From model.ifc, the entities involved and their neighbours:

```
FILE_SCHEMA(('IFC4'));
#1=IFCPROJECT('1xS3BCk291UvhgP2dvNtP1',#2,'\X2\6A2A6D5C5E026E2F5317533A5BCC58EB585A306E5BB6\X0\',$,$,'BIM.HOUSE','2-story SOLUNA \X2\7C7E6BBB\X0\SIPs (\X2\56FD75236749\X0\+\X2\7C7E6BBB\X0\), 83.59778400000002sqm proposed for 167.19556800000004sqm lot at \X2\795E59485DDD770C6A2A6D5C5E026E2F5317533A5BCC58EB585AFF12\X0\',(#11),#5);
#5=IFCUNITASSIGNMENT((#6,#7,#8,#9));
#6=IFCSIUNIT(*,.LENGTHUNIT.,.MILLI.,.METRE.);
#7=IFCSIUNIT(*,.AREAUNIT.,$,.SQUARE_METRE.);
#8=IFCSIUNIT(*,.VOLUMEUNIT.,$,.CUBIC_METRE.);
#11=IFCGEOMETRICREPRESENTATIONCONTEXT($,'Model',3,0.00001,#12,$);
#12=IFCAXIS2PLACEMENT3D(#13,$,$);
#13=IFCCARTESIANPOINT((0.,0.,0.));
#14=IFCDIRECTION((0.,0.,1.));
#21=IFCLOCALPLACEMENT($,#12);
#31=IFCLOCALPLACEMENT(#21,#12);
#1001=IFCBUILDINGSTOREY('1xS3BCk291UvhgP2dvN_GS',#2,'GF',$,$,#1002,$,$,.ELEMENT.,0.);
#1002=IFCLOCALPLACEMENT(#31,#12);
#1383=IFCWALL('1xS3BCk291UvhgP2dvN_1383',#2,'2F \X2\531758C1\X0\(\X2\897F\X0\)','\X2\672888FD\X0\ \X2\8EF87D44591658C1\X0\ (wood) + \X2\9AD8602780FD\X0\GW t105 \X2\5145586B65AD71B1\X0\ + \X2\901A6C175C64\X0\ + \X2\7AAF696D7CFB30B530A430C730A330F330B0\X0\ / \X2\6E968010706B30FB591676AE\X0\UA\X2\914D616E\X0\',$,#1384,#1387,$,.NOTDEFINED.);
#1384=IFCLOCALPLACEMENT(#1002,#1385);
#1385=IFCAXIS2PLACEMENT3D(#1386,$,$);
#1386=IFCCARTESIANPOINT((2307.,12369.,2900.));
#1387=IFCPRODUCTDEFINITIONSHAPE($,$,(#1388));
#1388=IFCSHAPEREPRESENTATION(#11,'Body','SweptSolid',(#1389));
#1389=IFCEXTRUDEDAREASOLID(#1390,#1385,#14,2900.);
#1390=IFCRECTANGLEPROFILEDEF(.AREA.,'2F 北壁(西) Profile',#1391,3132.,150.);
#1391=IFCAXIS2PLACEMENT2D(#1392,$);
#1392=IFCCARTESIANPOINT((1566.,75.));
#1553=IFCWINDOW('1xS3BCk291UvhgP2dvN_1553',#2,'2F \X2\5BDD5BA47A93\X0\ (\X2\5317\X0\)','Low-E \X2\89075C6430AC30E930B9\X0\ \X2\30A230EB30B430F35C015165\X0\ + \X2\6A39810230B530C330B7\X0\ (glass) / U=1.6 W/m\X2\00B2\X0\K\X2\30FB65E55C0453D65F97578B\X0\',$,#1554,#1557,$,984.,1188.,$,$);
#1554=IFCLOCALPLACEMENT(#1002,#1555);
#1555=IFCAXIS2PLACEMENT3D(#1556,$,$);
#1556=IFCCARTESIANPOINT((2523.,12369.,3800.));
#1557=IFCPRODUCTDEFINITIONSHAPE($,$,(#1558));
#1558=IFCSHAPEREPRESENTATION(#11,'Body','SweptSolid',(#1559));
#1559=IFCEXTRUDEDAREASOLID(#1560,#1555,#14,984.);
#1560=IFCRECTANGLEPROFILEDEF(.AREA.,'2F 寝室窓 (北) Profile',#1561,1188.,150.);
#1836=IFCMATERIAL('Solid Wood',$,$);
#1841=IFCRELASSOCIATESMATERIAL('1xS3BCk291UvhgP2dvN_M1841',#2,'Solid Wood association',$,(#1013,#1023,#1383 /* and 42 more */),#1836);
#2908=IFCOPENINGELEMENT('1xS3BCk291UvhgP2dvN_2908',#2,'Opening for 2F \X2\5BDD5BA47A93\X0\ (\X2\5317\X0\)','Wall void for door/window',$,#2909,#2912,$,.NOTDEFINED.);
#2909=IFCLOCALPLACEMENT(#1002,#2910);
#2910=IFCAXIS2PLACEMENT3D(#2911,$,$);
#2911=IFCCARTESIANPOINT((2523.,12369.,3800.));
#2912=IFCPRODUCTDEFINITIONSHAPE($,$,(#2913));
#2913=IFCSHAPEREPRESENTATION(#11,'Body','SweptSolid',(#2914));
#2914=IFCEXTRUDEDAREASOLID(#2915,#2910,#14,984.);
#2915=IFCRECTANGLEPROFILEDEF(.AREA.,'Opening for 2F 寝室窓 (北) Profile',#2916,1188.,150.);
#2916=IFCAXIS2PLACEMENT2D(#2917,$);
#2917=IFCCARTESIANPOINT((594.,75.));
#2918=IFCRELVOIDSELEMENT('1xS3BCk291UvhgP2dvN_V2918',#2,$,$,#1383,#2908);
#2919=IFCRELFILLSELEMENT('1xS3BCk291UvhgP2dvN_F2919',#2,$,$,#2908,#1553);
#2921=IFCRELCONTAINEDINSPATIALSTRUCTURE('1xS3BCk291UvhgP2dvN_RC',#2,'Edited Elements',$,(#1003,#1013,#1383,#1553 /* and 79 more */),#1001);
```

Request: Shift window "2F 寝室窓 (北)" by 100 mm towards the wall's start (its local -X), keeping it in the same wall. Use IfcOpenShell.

```python
import ifcopenshell
import ifcopenshell.api.geometry
import ifcopenshell.util.placement
import ifcopenshell.util.unit

model = ifcopenshell.open("model.ifc")
unit_scale = ifcopenshell.util.unit.calculate_unit_scale(model)

window = model.by_guid("1xS3BCk291UvhgP2dvN_1553")
opening = window.FillsVoids[0].RelatingOpeningElement
wall = opening.VoidsElements[0].RelatingBuildingElement

wall_matrix = ifcopenshell.util.placement.get_local_placement(wall.ObjectPlacement)
shift = wall_matrix[:3, 0] * -0.1 / unit_scale
before = ifcopenshell.util.placement.get_local_placement(window.ObjectPlacement)[:3, 3].copy()

# The window is not placed relative to its opening, so move both.
for product in (opening, window):
    matrix = ifcopenshell.util.placement.get_local_placement(product.ObjectPlacement)
    matrix[:3, 3] += shift
    ifcopenshell.api.geometry.edit_object_placement(model, product=product, matrix=matrix, is_si=False)

after = ifcopenshell.util.placement.get_local_placement(window.ObjectPlacement)[:3, 3]
print("window moved by", (after - before).round(3) + 0.0)

model.write("model_v2.ifc")
```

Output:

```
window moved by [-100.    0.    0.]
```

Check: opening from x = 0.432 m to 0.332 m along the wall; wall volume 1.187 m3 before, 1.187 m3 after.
